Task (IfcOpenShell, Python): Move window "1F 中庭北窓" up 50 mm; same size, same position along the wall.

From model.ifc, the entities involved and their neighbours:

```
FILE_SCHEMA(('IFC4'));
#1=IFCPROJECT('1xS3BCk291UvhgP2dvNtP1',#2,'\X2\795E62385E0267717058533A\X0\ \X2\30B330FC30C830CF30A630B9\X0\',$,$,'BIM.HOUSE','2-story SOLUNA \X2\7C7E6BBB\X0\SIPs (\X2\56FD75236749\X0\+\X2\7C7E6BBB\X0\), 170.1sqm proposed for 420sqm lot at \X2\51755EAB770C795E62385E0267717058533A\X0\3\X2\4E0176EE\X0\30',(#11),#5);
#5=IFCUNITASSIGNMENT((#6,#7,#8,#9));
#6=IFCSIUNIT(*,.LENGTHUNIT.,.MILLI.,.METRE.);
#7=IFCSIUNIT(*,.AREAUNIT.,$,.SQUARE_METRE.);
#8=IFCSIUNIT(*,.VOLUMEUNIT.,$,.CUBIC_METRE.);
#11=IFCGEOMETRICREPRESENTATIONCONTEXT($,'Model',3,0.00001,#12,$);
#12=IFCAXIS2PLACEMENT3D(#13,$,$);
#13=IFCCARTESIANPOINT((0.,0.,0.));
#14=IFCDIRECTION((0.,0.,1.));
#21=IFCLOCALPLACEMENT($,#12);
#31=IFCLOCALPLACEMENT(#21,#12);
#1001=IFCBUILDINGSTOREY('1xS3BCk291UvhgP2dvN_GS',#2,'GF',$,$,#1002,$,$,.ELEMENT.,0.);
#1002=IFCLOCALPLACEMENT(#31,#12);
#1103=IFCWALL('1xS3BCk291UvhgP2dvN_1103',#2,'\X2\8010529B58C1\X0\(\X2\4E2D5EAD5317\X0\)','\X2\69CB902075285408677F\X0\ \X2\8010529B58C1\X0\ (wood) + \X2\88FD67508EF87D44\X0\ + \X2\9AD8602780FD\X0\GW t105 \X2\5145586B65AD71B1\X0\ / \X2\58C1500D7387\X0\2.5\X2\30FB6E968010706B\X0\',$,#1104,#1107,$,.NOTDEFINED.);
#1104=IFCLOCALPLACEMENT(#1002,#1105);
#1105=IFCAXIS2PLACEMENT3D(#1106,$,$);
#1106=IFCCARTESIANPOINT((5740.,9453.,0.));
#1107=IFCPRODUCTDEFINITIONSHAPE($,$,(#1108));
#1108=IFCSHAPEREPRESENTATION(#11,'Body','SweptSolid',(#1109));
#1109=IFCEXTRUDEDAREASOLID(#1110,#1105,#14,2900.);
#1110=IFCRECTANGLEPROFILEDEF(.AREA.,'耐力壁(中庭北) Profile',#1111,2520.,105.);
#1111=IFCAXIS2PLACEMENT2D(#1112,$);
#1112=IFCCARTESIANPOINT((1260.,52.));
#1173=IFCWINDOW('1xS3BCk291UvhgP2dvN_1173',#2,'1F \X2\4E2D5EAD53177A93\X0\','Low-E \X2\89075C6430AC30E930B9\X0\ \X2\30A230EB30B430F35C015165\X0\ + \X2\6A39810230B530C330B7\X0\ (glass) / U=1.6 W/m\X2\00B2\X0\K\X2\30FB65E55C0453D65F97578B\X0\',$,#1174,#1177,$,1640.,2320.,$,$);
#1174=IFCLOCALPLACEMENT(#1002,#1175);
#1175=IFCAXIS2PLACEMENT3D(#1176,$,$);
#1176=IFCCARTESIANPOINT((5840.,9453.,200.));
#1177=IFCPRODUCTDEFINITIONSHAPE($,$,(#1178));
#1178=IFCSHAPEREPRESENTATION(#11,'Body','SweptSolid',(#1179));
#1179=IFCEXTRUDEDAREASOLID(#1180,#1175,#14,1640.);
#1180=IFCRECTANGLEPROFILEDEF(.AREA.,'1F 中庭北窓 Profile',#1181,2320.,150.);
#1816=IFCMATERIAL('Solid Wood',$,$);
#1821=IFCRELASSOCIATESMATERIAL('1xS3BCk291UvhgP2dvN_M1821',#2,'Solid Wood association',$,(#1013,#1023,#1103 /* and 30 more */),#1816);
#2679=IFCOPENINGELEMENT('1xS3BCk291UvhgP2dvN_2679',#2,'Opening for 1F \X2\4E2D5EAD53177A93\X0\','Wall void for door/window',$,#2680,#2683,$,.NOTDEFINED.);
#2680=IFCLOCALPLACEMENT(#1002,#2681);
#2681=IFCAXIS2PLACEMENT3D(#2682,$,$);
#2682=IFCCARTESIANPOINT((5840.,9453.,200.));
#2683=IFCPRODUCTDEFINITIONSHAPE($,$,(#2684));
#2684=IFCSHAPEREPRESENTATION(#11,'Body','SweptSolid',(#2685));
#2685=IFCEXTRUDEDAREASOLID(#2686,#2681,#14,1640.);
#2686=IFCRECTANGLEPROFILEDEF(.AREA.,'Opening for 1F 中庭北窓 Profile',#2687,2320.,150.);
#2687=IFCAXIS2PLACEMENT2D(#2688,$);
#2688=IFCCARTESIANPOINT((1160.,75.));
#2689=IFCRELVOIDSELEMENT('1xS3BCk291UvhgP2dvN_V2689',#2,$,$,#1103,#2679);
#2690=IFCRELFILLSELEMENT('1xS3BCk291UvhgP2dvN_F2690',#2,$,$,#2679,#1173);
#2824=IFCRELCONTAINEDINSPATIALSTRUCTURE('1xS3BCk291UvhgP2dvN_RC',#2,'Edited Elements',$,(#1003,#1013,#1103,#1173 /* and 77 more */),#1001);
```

```python
import numpy as np
import ifcopenshell
import ifcopenshell.api.geometry
import ifcopenshell.util.placement
import ifcopenshell.util.unit

model = ifcopenshell.open("model.ifc")
unit_scale = ifcopenshell.util.unit.calculate_unit_scale(model)

window = model.by_guid("1xS3BCk291UvhgP2dvN_1173")
opening = window.FillsVoids[0].RelatingOpeningElement
dz = 0.05 / unit_scale

shift = np.array([0.0, 0.0, dz])
# The window is not placed relative to its opening, so move both.
for product in (opening, window):
    matrix = ifcopenshell.util.placement.get_local_placement(product.ObjectPlacement)
    matrix[:3, 3] += shift
    ifcopenshell.api.geometry.edit_object_placement(model, product=product, matrix=matrix, is_si=False)

print(f"moved by {dz * unit_scale:+.3f} m")

model.write("model_v2.ifc")
```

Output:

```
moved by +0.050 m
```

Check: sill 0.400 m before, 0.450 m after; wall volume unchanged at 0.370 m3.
